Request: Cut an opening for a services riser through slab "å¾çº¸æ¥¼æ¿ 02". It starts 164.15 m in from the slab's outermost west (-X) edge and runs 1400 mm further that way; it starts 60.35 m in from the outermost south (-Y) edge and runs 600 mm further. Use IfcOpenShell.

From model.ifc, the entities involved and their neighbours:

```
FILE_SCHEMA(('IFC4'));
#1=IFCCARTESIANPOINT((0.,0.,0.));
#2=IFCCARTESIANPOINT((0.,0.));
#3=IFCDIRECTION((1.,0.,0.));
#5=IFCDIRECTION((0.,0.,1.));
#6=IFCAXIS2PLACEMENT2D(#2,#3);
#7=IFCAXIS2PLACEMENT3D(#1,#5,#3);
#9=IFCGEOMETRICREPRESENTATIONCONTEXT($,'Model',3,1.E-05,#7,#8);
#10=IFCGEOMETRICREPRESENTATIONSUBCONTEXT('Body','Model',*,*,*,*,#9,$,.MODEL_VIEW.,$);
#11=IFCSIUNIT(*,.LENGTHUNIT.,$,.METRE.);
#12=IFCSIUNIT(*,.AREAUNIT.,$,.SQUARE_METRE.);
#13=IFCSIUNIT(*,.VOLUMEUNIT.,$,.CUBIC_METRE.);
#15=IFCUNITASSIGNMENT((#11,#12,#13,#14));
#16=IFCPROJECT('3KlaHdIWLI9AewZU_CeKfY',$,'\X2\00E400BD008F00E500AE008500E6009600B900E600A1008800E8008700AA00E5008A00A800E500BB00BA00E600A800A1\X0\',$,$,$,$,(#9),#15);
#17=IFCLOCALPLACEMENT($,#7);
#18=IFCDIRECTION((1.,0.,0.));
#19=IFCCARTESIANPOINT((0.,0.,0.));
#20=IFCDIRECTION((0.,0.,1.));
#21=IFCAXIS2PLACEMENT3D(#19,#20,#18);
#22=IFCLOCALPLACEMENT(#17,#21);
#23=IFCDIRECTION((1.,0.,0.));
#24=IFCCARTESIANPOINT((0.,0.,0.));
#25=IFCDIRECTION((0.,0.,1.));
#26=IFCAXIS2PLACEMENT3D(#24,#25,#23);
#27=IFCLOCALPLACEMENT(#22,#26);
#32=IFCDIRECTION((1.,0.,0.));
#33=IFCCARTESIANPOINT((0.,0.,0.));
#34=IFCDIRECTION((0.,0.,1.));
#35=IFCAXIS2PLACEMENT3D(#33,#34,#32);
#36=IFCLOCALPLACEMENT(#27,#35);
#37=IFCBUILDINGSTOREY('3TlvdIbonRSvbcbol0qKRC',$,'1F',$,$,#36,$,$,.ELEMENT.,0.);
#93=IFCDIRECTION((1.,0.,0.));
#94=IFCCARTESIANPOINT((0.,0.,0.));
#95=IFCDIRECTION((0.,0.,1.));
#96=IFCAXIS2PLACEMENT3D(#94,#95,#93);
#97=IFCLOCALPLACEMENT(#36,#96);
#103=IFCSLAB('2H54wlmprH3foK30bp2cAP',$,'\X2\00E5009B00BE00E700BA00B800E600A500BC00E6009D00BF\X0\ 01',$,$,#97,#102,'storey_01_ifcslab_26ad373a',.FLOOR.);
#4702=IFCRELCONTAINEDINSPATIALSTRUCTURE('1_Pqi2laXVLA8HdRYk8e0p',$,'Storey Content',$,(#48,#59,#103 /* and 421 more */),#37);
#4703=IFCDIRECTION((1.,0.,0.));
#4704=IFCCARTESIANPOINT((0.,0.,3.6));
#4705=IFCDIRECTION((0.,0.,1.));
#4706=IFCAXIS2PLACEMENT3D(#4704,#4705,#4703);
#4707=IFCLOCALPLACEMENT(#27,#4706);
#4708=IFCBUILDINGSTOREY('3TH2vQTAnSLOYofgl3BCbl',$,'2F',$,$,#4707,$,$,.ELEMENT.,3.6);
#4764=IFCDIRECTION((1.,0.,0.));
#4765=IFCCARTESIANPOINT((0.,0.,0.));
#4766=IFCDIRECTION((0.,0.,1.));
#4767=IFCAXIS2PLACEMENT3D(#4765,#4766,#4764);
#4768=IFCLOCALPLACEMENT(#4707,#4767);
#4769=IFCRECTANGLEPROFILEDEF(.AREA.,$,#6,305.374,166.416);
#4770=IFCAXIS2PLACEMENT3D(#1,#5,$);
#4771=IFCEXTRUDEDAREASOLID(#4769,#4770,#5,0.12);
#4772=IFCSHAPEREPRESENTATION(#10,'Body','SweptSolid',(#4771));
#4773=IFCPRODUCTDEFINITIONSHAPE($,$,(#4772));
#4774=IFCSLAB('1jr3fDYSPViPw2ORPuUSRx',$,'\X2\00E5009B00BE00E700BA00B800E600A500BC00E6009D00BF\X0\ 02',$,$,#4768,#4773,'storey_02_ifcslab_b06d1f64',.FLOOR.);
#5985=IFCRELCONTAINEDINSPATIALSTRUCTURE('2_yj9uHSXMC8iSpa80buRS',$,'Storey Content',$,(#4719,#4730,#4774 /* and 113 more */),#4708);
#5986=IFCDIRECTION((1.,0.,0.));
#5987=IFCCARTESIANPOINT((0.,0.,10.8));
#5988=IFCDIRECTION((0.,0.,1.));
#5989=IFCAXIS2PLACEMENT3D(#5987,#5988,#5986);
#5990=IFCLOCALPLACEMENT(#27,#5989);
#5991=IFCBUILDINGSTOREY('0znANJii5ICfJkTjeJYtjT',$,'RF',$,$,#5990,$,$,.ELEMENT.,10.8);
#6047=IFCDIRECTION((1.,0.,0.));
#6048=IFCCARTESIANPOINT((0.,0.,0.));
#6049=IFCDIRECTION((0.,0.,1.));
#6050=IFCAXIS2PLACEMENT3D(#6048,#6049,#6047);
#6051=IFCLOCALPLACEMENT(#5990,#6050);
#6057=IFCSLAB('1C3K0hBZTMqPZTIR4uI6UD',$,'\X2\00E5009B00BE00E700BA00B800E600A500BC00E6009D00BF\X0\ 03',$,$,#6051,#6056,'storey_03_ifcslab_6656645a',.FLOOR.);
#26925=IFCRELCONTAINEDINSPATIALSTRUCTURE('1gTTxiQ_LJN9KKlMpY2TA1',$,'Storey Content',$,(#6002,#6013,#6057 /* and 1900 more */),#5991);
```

```python
import numpy as np
import ifcopenshell
import ifcopenshell.api.feature
import ifcopenshell.api.geometry
import ifcopenshell.api.root
import ifcopenshell.geom
import ifcopenshell.util.placement
import ifcopenshell.util.representation
import ifcopenshell.util.shape
import ifcopenshell.util.unit

model = ifcopenshell.open("model.ifc")
unit_scale = ifcopenshell.util.unit.calculate_unit_scale(model)
settings = ifcopenshell.geom.settings()


def volume(element):
    """Net volume in cubic metres, openings subtracted."""
    shape = ifcopenshell.geom.create_shape(settings, element)
    return ifcopenshell.util.shape.get_volume(shape.geometry)


slab = model.by_id(4774)
before = volume(slab)

# Extent in the slab's own axes, in metres. The edges named are its -X and -Y sides.
slab_shape = ifcopenshell.geom.create_shape(settings, slab)
vertices = ifcopenshell.util.shape.get_vertices(slab_shape.geometry)
x_min, y_min, bottom = vertices.min(axis=0)
top = vertices[:, 2].max()

opening = ifcopenshell.api.root.create_entity(model, ifc_class="IfcOpeningElement", name="Services riser opening", predefined_type="OPENING")
context = ifcopenshell.util.representation.get_context(model, "Model", "Body", "MODEL_VIEW")
width, depth = 1.4, 0.6
outline = [(0.0, 0.0), (width, 0.0), (width, depth), (0.0, depth), (0.0, 0.0)]
# Overshoot both faces by 50 mm so the cut is clean.
shape = ifcopenshell.api.geometry.add_slab_representation(
    model, context=context, depth=top - bottom + 0.1, polyline=outline
)
ifcopenshell.api.geometry.assign_representation(model, product=opening, representation=shape)

matrix = ifcopenshell.util.placement.get_local_placement(slab.ObjectPlacement)
matrix[:, 3] = matrix @ np.append(np.array([x_min + 164.15, y_min + 60.35, bottom - 0.05]) / unit_scale, 1.0)
ifcopenshell.api.geometry.edit_object_placement(model, product=opening, matrix=matrix, is_si=False)
ifcopenshell.api.feature.add_feature(model, feature=opening, element=slab)

after = volume(slab)

print(f"slab volume {before:.3f} -> {after:.3f} m3")

model.write("model_rev.ifc")
```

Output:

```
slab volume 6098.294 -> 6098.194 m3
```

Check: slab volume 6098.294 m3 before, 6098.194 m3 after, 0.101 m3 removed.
